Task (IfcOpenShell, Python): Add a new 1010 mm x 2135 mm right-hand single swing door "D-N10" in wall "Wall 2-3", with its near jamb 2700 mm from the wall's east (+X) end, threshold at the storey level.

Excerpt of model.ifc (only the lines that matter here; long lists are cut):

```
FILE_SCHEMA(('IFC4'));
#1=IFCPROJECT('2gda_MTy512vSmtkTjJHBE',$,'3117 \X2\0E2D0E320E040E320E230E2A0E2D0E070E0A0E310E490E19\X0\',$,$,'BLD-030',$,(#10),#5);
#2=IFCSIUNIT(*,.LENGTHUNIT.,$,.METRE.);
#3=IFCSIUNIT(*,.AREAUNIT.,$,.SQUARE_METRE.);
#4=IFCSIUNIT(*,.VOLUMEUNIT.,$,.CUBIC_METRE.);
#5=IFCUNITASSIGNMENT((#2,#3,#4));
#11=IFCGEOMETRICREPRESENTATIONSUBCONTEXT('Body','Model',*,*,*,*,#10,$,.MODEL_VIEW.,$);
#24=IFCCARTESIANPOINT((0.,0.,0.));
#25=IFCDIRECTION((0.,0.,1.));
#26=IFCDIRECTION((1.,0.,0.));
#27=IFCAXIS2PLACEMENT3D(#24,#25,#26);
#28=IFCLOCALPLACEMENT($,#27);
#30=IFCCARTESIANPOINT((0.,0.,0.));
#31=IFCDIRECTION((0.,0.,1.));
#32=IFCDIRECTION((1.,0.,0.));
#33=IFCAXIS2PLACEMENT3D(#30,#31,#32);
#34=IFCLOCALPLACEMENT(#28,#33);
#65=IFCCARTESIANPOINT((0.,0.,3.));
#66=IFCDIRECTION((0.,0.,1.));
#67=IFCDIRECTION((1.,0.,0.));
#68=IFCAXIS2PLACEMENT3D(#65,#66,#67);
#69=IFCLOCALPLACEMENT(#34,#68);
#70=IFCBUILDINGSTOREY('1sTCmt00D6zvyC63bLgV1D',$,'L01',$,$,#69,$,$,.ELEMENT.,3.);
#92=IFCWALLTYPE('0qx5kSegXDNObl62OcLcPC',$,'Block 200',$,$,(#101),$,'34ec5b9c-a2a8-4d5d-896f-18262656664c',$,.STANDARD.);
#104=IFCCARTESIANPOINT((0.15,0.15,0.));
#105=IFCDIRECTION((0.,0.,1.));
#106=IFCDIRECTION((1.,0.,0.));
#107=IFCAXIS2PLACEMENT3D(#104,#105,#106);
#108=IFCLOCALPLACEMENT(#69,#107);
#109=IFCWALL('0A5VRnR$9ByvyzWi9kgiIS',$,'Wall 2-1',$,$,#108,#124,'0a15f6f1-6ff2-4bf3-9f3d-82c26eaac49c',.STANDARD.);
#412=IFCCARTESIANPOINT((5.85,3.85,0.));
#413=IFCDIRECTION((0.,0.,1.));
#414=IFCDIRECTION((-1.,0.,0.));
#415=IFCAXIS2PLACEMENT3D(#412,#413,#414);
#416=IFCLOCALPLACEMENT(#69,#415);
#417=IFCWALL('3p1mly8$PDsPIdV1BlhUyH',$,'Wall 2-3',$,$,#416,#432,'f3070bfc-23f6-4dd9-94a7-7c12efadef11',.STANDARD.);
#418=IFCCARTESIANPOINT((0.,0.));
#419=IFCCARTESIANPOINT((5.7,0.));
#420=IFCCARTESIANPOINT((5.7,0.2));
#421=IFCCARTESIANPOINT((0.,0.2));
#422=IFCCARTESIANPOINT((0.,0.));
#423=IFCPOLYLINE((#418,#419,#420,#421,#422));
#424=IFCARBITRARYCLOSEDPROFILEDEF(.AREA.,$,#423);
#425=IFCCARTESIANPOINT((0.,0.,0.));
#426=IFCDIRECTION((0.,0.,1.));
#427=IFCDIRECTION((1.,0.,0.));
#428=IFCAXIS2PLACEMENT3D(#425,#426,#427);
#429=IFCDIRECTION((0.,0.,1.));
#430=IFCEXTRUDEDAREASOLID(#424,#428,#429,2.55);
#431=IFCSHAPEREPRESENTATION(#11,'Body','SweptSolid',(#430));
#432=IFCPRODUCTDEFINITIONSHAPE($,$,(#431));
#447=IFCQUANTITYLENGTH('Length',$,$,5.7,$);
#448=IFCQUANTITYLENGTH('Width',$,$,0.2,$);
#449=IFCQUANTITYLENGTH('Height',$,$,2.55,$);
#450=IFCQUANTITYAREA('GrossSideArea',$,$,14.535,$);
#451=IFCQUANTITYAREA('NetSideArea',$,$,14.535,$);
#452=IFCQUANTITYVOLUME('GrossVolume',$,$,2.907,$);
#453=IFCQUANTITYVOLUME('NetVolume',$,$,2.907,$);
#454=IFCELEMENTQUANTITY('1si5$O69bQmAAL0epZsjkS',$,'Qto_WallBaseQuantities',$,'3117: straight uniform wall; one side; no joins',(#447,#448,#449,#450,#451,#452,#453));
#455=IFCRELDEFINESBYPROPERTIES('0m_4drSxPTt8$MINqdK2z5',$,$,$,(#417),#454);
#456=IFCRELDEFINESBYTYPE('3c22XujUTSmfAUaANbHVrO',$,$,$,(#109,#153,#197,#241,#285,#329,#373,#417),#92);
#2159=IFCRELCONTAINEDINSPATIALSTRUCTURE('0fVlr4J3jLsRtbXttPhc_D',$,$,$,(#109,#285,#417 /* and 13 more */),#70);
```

```python
import numpy as np
import ifcopenshell
import ifcopenshell.api.feature
import ifcopenshell.api.geometry
import ifcopenshell.api.pset
import ifcopenshell.api.root
import ifcopenshell.api.spatial
import ifcopenshell.geom
import ifcopenshell.util.element
import ifcopenshell.util.placement
import ifcopenshell.util.representation
import ifcopenshell.util.shape
import ifcopenshell.util.unit

model = ifcopenshell.open("model.ifc")
unit_scale = ifcopenshell.util.unit.calculate_unit_scale(model)
area_scale = ifcopenshell.util.unit.calculate_unit_scale(model, "AREAUNIT")
volume_scale = ifcopenshell.util.unit.calculate_unit_scale(model, "VOLUMEUNIT")
settings = ifcopenshell.geom.settings()


def volume(element):
    """Net volume in cubic metres, openings subtracted."""
    shape = ifcopenshell.geom.create_shape(settings, element)
    return ifcopenshell.util.shape.get_volume(shape.geometry)


wall = model.by_guid("3p1mly8$PDsPIdV1BlhUyH")
storey = ifcopenshell.util.element.get_container(wall, ifc_class="IfcBuildingStorey")
context = ifcopenshell.util.representation.get_context(model, "Model", "Body", "MODEL_VIEW")
before = volume(wall)

width, height, from_end, sill = 1.01, 2.135, 2.7, 0.0  # metres

# The wall runs along its own X axis, and the end named is its -X end.
wall_shape = ifcopenshell.geom.create_shape(settings, wall)
x, y, z = ifcopenshell.util.shape.get_vertices(wall_shape.geometry).T
start = x.min() + from_end
face, thickness = float(y.min()), float(y.max() - y.min())
wall_matrix = ifcopenshell.util.placement.get_local_placement(wall.ObjectPlacement)
level = ifcopenshell.util.placement.get_local_placement(storey.ObjectPlacement)[2, 3]


def in_wall(x, y):
    """Placement at x, y metres in the wall's axes, at sill height."""
    matrix = wall_matrix.copy()
    matrix[:, 3] = wall_matrix @ np.array([x / unit_scale, y / unit_scale, 0.0, 1.0])
    matrix[2, 3] = level + sill / unit_scale
    return matrix


# Opening: a box that overshoots both wall faces by 50 mm.
opening = ifcopenshell.api.root.create_entity(model, ifc_class="IfcOpeningElement", predefined_type="OPENING")
box = ifcopenshell.api.geometry.add_wall_representation(
    model, context=context, length=width, height=height, thickness=thickness + 0.1
)
ifcopenshell.api.geometry.assign_representation(model, product=opening, representation=box)
ifcopenshell.api.geometry.edit_object_placement(model, product=opening, matrix=in_wall(start, face - 0.05), is_si=False)
ifcopenshell.api.feature.add_feature(model, feature=opening, element=wall)

door = ifcopenshell.api.root.create_entity(model, ifc_class="IfcDoor", name="D-N10", predefined_type="DOOR")
door.OverallWidth, door.OverallHeight = width / unit_scale, height / unit_scale
door.OperationType = "SINGLE_SWING_RIGHT"
body = ifcopenshell.api.geometry.add_door_representation(
    model,
    context=context,
    overall_width=door.OverallWidth,
    overall_height=door.OverallHeight,
    operation_type="SINGLE_SWING_RIGHT",
    lining_properties={"LiningDepth": thickness / unit_scale, "ThresholdDepth": thickness / unit_scale},
)
ifcopenshell.api.geometry.assign_representation(model, product=door, representation=body)
ifcopenshell.api.spatial.assign_container(model, products=[door], relating_structure=storey)
ifcopenshell.api.feature.add_filling(model, opening=opening, element=door)

# The lining spans the wall, so the door starts at the wall face.
ifcopenshell.api.geometry.edit_object_placement(model, product=door, matrix=in_wall(start, face), is_si=False)

after = volume(wall)

# Update the wall's stored quantities.
qto = model.by_id(ifcopenshell.util.element.get_pset(wall, "Qto_WallBaseQuantities", should_inherit=False)["id"])
ifcopenshell.api.pset.edit_qto(model, qto=qto, properties={
    "NetSideArea": after / thickness / area_scale,
    "NetVolume": after / volume_scale,
})

print(f"wall volume {before:.3f} -> {after:.3f} m3")

model.write("model-out.ifc")
```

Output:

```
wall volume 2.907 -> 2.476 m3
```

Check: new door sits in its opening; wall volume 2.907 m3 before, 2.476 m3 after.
